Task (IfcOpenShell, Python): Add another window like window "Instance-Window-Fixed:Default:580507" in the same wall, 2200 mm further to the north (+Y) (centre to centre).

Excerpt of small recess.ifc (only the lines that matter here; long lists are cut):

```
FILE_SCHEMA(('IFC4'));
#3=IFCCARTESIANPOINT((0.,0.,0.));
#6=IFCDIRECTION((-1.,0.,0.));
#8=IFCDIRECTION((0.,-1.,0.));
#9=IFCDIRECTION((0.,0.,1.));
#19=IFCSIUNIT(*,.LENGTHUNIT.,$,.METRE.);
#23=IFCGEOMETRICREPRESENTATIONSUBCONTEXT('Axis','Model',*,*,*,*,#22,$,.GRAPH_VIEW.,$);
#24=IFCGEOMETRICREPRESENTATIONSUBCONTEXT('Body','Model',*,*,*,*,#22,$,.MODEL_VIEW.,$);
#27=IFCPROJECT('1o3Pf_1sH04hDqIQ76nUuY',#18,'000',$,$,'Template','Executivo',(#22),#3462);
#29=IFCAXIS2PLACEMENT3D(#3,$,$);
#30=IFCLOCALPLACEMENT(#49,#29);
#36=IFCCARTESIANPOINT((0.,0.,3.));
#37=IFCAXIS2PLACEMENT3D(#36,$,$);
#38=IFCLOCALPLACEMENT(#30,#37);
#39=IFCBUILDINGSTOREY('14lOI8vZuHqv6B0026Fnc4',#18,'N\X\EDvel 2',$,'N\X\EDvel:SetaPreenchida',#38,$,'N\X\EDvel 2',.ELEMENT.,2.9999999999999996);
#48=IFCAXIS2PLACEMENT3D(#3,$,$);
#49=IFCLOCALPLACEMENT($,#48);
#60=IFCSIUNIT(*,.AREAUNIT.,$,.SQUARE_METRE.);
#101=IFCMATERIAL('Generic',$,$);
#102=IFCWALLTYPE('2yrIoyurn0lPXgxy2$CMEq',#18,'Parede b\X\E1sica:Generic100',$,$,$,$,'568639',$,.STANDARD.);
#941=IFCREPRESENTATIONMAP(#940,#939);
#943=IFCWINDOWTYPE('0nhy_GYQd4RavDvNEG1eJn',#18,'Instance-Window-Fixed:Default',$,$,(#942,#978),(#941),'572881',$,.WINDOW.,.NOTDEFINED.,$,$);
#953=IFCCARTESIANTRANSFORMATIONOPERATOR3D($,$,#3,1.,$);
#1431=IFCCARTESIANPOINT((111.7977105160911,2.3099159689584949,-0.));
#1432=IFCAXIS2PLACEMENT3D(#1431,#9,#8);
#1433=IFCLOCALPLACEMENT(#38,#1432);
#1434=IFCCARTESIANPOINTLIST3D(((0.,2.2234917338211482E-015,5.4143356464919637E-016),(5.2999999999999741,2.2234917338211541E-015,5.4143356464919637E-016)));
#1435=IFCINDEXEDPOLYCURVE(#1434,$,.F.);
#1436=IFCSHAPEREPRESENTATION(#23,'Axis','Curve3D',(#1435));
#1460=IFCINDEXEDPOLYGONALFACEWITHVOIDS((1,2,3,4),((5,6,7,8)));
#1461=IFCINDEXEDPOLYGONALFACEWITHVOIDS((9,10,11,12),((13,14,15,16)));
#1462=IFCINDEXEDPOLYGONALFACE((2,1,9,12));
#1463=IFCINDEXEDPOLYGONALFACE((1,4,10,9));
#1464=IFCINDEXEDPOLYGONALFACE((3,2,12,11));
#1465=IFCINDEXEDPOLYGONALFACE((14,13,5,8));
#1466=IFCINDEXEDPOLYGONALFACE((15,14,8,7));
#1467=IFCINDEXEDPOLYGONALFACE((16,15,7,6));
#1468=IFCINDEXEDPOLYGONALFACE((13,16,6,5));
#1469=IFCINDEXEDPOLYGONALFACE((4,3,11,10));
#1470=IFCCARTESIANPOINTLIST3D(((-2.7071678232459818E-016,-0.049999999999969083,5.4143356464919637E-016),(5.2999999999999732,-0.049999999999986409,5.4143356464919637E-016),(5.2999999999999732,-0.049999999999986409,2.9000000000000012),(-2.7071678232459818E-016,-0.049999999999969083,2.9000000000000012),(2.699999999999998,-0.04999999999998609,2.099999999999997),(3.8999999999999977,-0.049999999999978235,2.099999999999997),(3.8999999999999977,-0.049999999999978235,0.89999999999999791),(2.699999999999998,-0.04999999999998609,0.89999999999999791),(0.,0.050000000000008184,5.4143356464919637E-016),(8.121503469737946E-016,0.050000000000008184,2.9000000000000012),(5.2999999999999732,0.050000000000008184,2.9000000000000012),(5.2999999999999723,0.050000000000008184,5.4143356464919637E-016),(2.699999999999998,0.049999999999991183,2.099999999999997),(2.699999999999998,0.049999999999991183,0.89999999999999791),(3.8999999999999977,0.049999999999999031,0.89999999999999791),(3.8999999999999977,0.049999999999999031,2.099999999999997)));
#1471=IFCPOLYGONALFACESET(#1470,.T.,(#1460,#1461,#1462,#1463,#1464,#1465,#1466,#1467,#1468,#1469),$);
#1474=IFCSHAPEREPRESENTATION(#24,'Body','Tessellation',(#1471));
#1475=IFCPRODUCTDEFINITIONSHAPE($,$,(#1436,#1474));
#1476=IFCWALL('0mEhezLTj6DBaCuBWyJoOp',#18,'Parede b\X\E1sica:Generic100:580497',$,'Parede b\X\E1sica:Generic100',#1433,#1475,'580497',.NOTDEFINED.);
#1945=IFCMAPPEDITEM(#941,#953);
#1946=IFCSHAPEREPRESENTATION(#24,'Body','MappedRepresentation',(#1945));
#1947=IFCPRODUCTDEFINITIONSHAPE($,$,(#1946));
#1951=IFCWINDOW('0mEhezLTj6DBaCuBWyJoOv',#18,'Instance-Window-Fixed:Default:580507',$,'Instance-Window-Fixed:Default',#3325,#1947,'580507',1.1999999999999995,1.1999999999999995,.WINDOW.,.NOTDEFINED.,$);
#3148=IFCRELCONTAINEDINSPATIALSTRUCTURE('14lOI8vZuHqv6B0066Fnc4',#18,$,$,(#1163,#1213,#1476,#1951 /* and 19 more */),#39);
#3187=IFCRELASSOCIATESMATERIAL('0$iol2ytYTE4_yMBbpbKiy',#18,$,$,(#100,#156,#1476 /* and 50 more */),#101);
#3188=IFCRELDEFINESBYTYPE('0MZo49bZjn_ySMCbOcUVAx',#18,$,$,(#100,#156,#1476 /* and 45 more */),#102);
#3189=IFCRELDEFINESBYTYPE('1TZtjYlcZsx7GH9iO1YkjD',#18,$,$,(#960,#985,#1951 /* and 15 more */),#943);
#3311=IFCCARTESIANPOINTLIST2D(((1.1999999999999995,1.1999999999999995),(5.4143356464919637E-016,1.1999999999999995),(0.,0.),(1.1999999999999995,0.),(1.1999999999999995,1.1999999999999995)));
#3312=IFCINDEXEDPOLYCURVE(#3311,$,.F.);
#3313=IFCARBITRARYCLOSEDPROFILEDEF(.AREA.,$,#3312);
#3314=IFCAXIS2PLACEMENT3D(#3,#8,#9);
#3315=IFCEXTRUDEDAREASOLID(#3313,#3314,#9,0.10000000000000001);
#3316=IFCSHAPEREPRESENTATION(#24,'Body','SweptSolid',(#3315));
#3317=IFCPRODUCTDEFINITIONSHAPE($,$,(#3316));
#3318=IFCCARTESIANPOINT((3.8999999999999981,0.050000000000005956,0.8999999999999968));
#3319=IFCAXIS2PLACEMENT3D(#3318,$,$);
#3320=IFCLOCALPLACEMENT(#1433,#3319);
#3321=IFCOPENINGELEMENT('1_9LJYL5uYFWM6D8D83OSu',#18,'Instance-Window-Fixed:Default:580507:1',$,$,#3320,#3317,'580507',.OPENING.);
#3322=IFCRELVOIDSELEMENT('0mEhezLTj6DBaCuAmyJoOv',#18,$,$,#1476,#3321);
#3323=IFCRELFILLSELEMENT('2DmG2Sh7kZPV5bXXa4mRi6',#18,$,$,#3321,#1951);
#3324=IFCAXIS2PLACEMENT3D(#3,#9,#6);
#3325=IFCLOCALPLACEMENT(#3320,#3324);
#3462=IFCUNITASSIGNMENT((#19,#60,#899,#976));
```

```python
import ifcopenshell
import ifcopenshell.api.feature
import ifcopenshell.api.geometry
import ifcopenshell.api.root
import ifcopenshell.geom
import ifcopenshell.util.element
import ifcopenshell.util.placement
import ifcopenshell.util.shape
import ifcopenshell.util.unit

model = ifcopenshell.open("small recess.ifc")
unit_scale = ifcopenshell.util.unit.calculate_unit_scale(model)
settings = ifcopenshell.geom.settings()


def volume(element):
    """Net volume in cubic metres, openings subtracted."""
    shape = ifcopenshell.geom.create_shape(settings, element)
    return ifcopenshell.util.shape.get_volume(shape.geometry)


def reuse_history(source, copy):
    """copy_class also copies each property set's owner history, people and application; keep the originals."""
    for rel in copy.IsDefinedBy:
        if rel.is_a("IfcRelDefinesByProperties") and (history := rel.RelatingPropertyDefinition.OwnerHistory):
            rel.RelatingPropertyDefinition.OwnerHistory = source.OwnerHistory
            ifcopenshell.util.element.remove_deep2(model, history)


window = model.by_guid("0mEhezLTj6DBaCuBWyJoOv")
opening = window.FillsVoids[0].RelatingOpeningElement
wall = opening.VoidsElements[0].RelatingBuildingElement
before = volume(wall)
shift = ifcopenshell.util.placement.get_local_placement(wall.ObjectPlacement)[:3, 0] * -2.2 / unit_scale

# copy_class copies the void relationship, type, container and properties, but no geometry.
new_opening = ifcopenshell.api.root.copy_class(model, product=opening)
new_opening.Representation = ifcopenshell.util.element.copy_deep(
    model, opening.Representation, exclude=["IfcGeometricRepresentationContext", "IfcRepresentationMap"]
)
new_opening.Name = "Instance-Window-Fixed:Default"
new_opening.Tag = None
new_window = ifcopenshell.api.root.copy_class(model, product=window)
new_window.Representation = ifcopenshell.util.element.copy_deep(
    model, window.Representation, exclude=["IfcGeometricRepresentationContext", "IfcRepresentationMap"]
)
new_window.Name = "Instance-Window-Fixed:Default"
new_window.Tag = None
reuse_history(window, new_window)
ifcopenshell.api.feature.add_filling(model, opening=new_opening, element=new_window)

for old, new in ((opening, new_opening), (window, new_window)):
    matrix = ifcopenshell.util.placement.get_local_placement(old.ObjectPlacement)
    matrix[:3, 3] += shift
    ifcopenshell.api.geometry.edit_object_placement(model, product=new, matrix=matrix, is_si=False)

after = volume(wall)

print(f"wall volume {before:.3f} -> {after:.3f} m3")

model.write("small recess_rev.ifc")
```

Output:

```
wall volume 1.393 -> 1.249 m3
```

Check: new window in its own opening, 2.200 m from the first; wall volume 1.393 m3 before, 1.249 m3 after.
